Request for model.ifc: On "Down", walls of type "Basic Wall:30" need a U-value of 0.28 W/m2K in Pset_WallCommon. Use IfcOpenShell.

First a look at what the model holds.

```python
import ifcopenshell
import ifcopenshell.util.element

model = ifcopenshell.open("model.ifc")
print(model.schema)
storey = next(s for s in model.by_type("IfcBuildingStorey") if s.Name == "Down")
walls = [e for e in ifcopenshell.util.element.get_decomposition(storey) if e.is_a("IfcWall")]
seen = {}
for e in walls:
    element_type = ifcopenshell.util.element.get_type(e)
    key = (element_type.Name if element_type != e and element_type else None, ifcopenshell.util.element.get_pset(e, "Pset_WallCommon", "ThermalTransmittance"))
    seen[key] = seen.get(key, 0) + 1
for (name, value), count in sorted(seen.items(), key=str):
    print(count, "x", name, "|", value)
```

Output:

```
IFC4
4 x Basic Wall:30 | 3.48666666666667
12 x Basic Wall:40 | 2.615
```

```python
import ifcopenshell
import ifcopenshell.api.pset
import ifcopenshell.util.element

model = ifcopenshell.open("model.ifc")

storey = next(s for s in model.by_type("IfcBuildingStorey") if s.Name == "Down")
walls = [e for e in ifcopenshell.util.element.get_decomposition(storey) if e.is_a("IfcWall")]

count = 0
for e in walls:
    element_type = ifcopenshell.util.element.get_type(e)
    if element_type in (None, e) or element_type.Name != "Basic Wall:30":
        continue
    # add_pset returns the element's existing set when there is one.
    pset = ifcopenshell.api.pset.add_pset(model, product=e, name="Pset_WallCommon")
    ifcopenshell.api.pset.edit_pset(model, pset=pset, properties={"ThermalTransmittance": 0.28})
    count += 1

print(count, "walls updated")

model.write("model_updated.ifc")
```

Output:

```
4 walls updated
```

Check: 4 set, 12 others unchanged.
